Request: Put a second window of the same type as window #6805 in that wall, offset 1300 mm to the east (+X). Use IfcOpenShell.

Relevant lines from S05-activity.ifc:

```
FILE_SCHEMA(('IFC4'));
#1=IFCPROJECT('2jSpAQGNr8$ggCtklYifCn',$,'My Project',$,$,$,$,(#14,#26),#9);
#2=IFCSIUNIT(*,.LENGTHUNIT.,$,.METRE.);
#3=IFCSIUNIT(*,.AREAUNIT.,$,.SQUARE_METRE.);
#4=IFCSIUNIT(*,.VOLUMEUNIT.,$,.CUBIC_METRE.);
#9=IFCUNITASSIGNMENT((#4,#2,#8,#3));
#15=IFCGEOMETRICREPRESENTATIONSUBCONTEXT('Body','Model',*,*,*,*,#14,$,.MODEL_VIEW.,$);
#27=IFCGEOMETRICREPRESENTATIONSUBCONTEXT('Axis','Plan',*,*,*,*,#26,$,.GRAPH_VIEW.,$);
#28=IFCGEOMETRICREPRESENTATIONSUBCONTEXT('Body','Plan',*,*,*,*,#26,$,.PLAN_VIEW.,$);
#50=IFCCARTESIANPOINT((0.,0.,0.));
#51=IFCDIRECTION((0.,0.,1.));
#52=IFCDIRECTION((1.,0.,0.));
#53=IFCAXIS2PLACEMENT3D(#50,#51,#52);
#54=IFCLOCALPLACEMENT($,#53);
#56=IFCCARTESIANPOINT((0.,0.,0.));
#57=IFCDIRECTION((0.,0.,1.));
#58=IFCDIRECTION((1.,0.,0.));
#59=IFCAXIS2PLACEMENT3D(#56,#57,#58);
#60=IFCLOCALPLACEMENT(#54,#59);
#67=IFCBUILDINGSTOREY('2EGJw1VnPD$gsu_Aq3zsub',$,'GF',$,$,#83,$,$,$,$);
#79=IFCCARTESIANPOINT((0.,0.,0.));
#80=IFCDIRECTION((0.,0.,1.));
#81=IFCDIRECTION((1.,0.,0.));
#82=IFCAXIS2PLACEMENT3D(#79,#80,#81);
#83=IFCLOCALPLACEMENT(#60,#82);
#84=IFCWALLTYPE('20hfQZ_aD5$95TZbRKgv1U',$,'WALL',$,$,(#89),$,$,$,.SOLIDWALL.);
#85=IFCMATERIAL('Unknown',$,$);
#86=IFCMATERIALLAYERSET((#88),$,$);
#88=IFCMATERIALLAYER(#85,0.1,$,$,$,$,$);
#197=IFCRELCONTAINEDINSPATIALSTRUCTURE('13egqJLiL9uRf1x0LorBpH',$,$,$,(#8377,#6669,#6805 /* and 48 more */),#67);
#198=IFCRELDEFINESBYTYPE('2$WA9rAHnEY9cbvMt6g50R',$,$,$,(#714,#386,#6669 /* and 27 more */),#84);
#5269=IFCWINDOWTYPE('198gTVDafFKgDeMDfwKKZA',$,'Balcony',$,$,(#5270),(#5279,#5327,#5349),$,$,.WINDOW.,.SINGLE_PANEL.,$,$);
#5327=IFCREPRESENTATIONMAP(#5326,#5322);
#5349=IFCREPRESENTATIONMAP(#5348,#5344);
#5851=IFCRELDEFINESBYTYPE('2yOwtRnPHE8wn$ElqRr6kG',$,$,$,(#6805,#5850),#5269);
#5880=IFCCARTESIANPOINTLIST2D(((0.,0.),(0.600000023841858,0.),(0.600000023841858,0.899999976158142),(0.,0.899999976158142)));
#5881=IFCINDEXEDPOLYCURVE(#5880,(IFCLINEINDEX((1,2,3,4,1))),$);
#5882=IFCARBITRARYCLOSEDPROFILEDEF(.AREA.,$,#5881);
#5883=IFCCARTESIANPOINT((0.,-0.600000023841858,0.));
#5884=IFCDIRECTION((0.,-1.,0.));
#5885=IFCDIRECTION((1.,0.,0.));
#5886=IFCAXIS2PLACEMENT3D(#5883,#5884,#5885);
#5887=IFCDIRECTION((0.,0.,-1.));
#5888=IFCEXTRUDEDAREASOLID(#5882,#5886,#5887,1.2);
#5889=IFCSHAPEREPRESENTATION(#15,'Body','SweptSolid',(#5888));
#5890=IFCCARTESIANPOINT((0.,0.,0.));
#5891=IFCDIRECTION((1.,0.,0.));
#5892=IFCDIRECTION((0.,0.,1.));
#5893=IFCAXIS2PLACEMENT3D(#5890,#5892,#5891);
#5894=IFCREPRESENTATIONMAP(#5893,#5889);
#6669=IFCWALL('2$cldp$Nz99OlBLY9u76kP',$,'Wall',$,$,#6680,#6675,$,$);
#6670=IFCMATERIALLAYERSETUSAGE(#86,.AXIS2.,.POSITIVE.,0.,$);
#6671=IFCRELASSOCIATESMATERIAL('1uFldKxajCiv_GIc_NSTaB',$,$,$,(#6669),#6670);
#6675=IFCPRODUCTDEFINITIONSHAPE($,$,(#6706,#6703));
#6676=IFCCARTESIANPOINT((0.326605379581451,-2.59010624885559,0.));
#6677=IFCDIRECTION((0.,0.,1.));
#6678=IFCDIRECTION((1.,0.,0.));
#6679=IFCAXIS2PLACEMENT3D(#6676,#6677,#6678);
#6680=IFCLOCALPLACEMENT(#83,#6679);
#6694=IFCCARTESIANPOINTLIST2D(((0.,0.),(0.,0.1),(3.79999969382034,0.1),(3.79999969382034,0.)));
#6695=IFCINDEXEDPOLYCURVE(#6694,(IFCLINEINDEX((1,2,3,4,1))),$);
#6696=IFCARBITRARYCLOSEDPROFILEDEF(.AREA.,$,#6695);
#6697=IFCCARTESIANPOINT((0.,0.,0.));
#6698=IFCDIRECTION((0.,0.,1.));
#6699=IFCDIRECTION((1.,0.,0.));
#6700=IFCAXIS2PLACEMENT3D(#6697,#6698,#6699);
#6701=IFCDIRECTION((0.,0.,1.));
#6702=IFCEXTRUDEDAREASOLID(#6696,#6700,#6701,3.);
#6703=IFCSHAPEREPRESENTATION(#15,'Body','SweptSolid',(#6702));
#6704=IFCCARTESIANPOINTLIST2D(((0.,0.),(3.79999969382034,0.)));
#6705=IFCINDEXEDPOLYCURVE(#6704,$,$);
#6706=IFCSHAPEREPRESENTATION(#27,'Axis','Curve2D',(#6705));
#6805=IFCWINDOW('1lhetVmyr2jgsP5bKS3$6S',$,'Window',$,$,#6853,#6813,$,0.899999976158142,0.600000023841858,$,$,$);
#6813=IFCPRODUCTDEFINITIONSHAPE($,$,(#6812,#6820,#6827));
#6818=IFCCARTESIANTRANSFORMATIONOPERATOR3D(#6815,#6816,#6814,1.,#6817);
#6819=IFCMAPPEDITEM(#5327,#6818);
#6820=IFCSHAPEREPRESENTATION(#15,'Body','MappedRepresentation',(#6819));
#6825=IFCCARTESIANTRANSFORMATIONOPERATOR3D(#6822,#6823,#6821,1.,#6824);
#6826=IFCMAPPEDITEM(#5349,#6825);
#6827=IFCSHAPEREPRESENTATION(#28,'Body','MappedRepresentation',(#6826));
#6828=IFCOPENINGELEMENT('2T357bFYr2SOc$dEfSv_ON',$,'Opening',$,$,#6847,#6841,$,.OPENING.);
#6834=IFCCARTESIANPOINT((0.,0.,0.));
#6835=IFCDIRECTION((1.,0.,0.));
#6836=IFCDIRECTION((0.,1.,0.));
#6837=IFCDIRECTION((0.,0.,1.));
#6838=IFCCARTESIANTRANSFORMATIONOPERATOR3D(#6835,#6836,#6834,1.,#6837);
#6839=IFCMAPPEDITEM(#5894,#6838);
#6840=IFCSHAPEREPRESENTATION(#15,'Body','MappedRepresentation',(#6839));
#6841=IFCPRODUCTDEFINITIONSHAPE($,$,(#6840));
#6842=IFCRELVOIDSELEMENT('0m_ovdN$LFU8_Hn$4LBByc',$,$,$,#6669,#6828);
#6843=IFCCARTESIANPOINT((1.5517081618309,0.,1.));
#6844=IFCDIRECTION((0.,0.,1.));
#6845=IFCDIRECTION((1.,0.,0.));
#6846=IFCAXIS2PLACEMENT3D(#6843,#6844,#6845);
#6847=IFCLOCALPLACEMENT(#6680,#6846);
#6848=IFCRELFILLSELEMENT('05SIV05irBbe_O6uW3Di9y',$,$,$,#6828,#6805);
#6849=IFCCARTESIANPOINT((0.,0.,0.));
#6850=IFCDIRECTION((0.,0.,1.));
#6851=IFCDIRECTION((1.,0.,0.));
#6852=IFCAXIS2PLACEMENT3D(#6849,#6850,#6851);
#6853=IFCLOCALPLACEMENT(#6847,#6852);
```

```python
import ifcopenshell
import ifcopenshell.api.feature
import ifcopenshell.api.geometry
import ifcopenshell.api.root
import ifcopenshell.geom
import ifcopenshell.util.element
import ifcopenshell.util.placement
import ifcopenshell.util.shape
import ifcopenshell.util.unit

model = ifcopenshell.open("S05-activity.ifc")
unit_scale = ifcopenshell.util.unit.calculate_unit_scale(model)
settings = ifcopenshell.geom.settings()


def volume(element):
    """Net volume in cubic metres, openings subtracted."""
    shape = ifcopenshell.geom.create_shape(settings, element)
    return ifcopenshell.util.shape.get_volume(shape.geometry)


window = model.by_guid("1lhetVmyr2jgsP5bKS3$6S")
opening = window.FillsVoids[0].RelatingOpeningElement
wall = opening.VoidsElements[0].RelatingBuildingElement
before = volume(wall)
shift = ifcopenshell.util.placement.get_local_placement(wall.ObjectPlacement)[:3, 0] * 1.3 / unit_scale

# copy_class copies the void relationship, type, container and properties, but no geometry.
new_opening = ifcopenshell.api.root.copy_class(model, product=opening)
new_opening.Representation = ifcopenshell.util.element.copy_deep(
    model, opening.Representation, exclude=["IfcGeometricRepresentationContext", "IfcRepresentationMap"]
)
new_window = ifcopenshell.api.root.copy_class(model, product=window)
new_window.Representation = ifcopenshell.util.element.copy_deep(
    model, window.Representation, exclude=["IfcGeometricRepresentationContext", "IfcRepresentationMap"]
)
ifcopenshell.api.feature.add_filling(model, opening=new_opening, element=new_window)

for old, new in ((opening, new_opening), (window, new_window)):
    matrix = ifcopenshell.util.placement.get_local_placement(old.ObjectPlacement)
    matrix[:3, 3] += shift
    ifcopenshell.api.geometry.edit_object_placement(model, product=new, matrix=matrix, is_si=False)

after = volume(wall)

print(f"wall volume {before:.3f} -> {after:.3f} m3")

model.write("S05-activity_v2.ifc")
```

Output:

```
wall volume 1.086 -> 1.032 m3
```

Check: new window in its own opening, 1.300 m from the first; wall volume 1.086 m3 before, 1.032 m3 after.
